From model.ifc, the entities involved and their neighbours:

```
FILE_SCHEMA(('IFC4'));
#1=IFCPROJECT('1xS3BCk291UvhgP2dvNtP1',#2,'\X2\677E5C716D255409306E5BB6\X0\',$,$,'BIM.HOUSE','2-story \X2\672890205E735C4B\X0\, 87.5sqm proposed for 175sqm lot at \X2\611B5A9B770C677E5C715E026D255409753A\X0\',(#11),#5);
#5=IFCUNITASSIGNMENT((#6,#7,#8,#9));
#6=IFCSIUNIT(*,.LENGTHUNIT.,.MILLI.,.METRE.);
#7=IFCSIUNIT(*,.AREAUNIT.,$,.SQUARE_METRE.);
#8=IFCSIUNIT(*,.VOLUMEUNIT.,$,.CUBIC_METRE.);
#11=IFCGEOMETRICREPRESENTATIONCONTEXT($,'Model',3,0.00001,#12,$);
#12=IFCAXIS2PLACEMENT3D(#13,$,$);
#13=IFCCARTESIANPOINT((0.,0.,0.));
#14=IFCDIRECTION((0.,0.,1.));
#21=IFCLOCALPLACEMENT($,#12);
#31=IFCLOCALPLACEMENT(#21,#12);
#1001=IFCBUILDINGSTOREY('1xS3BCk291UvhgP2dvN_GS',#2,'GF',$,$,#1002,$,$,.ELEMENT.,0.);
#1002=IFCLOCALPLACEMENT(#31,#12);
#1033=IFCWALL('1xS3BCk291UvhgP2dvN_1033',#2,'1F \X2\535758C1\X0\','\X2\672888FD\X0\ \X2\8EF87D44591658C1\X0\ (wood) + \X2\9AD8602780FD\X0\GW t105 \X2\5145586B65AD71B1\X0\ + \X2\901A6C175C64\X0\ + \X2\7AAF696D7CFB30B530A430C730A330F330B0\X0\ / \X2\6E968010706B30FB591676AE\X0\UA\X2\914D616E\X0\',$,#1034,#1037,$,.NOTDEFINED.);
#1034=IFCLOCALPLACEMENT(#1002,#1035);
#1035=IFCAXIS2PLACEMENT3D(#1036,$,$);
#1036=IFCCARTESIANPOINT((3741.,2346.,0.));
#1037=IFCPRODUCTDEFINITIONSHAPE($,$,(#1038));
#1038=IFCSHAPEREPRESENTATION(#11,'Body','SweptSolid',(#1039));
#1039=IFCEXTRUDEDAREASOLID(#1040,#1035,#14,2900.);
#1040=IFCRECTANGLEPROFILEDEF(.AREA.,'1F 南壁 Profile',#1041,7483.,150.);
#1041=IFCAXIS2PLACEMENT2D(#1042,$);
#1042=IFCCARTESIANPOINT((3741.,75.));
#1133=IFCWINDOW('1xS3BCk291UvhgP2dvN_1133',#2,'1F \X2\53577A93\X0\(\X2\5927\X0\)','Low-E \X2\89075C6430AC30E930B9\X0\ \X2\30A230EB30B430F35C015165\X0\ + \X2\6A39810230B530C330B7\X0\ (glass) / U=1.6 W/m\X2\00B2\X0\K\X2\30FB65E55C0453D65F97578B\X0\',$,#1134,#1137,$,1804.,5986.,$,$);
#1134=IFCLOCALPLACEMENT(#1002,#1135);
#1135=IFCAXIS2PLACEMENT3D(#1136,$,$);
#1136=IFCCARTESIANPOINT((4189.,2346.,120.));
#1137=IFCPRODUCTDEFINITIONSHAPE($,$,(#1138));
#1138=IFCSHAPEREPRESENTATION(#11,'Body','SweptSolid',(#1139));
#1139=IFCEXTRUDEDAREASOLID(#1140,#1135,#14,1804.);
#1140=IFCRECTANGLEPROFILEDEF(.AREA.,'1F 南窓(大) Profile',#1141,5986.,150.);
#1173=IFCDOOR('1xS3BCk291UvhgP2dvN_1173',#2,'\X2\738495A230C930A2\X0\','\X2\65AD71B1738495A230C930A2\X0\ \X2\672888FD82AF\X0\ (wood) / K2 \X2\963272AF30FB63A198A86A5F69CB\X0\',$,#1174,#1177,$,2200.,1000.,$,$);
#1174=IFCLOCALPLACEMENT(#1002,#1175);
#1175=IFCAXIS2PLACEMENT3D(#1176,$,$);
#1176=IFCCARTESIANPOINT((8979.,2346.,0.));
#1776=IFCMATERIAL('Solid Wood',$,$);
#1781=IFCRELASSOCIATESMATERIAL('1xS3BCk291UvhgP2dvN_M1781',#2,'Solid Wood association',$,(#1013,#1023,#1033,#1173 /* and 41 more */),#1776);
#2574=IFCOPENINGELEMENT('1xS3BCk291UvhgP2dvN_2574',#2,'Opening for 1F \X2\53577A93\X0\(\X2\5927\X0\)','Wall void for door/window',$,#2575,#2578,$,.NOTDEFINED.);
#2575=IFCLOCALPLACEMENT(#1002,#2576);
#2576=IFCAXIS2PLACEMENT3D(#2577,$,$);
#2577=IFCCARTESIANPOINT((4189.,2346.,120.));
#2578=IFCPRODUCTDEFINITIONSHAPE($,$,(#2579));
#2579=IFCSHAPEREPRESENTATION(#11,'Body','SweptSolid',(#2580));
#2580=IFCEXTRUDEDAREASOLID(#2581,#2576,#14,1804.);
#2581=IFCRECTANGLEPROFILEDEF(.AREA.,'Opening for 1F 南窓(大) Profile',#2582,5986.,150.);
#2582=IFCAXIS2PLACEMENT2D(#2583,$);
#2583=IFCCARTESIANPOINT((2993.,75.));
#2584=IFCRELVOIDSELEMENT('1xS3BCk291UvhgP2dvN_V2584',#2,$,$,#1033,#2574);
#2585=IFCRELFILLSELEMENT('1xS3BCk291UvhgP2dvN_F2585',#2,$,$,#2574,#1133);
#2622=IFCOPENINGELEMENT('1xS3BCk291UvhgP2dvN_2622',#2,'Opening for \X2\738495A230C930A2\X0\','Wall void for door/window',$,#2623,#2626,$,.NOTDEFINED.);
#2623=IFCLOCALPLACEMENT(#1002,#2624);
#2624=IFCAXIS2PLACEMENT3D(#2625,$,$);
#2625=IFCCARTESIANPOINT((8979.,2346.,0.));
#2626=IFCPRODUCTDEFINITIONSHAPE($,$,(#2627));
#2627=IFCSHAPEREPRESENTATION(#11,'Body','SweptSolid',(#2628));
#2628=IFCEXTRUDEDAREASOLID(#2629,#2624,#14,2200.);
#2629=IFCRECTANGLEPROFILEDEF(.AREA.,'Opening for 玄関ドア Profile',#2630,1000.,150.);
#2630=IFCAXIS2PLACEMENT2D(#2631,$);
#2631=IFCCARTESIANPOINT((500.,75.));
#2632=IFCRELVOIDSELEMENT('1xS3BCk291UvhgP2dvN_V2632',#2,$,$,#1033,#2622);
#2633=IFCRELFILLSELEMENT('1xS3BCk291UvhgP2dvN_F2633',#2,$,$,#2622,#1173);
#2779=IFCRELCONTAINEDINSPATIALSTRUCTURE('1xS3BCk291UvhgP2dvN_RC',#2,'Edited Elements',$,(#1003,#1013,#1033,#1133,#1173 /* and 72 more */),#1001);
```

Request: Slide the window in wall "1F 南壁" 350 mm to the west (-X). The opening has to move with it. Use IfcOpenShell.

```python
import ifcopenshell
import ifcopenshell.api.geometry
import ifcopenshell.util.placement
import ifcopenshell.util.unit

model = ifcopenshell.open("model.ifc")
unit_scale = ifcopenshell.util.unit.calculate_unit_scale(model)

window = model.by_guid("1xS3BCk291UvhgP2dvN_1133")
opening = window.FillsVoids[0].RelatingOpeningElement
wall = opening.VoidsElements[0].RelatingBuildingElement

wall_matrix = ifcopenshell.util.placement.get_local_placement(wall.ObjectPlacement)
shift = wall_matrix[:3, 0] * -0.35 / unit_scale
before = ifcopenshell.util.placement.get_local_placement(window.ObjectPlacement)[:3, 3].copy()

# The window is not placed relative to its opening, so move both.
for product in (opening, window):
    matrix = ifcopenshell.util.placement.get_local_placement(product.ObjectPlacement)
    matrix[:3, 3] += shift
    ifcopenshell.api.geometry.edit_object_placement(model, product=product, matrix=matrix, is_si=False)

after = ifcopenshell.util.placement.get_local_placement(window.ObjectPlacement)[:3, 3]
print("window moved by", (after - before).round(3) + 0.0)

model.write("model_rev.ifc")
```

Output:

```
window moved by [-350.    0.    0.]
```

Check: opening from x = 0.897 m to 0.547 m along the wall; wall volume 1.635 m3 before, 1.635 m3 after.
